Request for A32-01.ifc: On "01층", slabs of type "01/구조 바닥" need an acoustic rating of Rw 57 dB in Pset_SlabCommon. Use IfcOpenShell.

First a look at what the model holds.

```python
import ifcopenshell
import ifcopenshell.util.element

model = ifcopenshell.open("A32-01.ifc")
print(model.schema)
storey = next(s for s in model.by_type("IfcBuildingStorey") if s.Name == "01층")
slabs = [e for e in ifcopenshell.util.element.get_decomposition(storey) if e.is_a("IfcSlab")]
seen = {}
for e in slabs:
    element_type = ifcopenshell.util.element.get_type(e)
    key = (element_type.Name if element_type != e and element_type else None, ifcopenshell.util.element.get_pset(e, "Pset_SlabCommon", "AcousticRating"))
    seen[key] = seen.get(key, 0) + 1
for (name, value), count in sorted(seen.items(), key=str):
    print(count, "x", name, "|", value)
```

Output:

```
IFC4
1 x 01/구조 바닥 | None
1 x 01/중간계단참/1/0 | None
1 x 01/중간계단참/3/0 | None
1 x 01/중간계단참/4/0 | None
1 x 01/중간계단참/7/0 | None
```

```python
import ifcopenshell
import ifcopenshell.api.pset
import ifcopenshell.util.element

model = ifcopenshell.open("A32-01.ifc")

storey = next(s for s in model.by_type("IfcBuildingStorey") if s.Name == "01층")
slabs = [e for e in ifcopenshell.util.element.get_decomposition(storey) if e.is_a("IfcSlab")]

count = 0
for e in slabs:
    element_type = ifcopenshell.util.element.get_type(e)
    if element_type in (None, e) or element_type.Name != "01/구조 바닥":
        continue
    # add_pset returns the element's existing set when there is one.
    pset = ifcopenshell.api.pset.add_pset(model, product=e, name="Pset_SlabCommon")
    ifcopenshell.api.pset.edit_pset(model, pset=pset, properties={"AcousticRating": "Rw 57 dB"})
    count += 1

print(count, "slabs updated")

model.write("A32-01_rev.ifc")
```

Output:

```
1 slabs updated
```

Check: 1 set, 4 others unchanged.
